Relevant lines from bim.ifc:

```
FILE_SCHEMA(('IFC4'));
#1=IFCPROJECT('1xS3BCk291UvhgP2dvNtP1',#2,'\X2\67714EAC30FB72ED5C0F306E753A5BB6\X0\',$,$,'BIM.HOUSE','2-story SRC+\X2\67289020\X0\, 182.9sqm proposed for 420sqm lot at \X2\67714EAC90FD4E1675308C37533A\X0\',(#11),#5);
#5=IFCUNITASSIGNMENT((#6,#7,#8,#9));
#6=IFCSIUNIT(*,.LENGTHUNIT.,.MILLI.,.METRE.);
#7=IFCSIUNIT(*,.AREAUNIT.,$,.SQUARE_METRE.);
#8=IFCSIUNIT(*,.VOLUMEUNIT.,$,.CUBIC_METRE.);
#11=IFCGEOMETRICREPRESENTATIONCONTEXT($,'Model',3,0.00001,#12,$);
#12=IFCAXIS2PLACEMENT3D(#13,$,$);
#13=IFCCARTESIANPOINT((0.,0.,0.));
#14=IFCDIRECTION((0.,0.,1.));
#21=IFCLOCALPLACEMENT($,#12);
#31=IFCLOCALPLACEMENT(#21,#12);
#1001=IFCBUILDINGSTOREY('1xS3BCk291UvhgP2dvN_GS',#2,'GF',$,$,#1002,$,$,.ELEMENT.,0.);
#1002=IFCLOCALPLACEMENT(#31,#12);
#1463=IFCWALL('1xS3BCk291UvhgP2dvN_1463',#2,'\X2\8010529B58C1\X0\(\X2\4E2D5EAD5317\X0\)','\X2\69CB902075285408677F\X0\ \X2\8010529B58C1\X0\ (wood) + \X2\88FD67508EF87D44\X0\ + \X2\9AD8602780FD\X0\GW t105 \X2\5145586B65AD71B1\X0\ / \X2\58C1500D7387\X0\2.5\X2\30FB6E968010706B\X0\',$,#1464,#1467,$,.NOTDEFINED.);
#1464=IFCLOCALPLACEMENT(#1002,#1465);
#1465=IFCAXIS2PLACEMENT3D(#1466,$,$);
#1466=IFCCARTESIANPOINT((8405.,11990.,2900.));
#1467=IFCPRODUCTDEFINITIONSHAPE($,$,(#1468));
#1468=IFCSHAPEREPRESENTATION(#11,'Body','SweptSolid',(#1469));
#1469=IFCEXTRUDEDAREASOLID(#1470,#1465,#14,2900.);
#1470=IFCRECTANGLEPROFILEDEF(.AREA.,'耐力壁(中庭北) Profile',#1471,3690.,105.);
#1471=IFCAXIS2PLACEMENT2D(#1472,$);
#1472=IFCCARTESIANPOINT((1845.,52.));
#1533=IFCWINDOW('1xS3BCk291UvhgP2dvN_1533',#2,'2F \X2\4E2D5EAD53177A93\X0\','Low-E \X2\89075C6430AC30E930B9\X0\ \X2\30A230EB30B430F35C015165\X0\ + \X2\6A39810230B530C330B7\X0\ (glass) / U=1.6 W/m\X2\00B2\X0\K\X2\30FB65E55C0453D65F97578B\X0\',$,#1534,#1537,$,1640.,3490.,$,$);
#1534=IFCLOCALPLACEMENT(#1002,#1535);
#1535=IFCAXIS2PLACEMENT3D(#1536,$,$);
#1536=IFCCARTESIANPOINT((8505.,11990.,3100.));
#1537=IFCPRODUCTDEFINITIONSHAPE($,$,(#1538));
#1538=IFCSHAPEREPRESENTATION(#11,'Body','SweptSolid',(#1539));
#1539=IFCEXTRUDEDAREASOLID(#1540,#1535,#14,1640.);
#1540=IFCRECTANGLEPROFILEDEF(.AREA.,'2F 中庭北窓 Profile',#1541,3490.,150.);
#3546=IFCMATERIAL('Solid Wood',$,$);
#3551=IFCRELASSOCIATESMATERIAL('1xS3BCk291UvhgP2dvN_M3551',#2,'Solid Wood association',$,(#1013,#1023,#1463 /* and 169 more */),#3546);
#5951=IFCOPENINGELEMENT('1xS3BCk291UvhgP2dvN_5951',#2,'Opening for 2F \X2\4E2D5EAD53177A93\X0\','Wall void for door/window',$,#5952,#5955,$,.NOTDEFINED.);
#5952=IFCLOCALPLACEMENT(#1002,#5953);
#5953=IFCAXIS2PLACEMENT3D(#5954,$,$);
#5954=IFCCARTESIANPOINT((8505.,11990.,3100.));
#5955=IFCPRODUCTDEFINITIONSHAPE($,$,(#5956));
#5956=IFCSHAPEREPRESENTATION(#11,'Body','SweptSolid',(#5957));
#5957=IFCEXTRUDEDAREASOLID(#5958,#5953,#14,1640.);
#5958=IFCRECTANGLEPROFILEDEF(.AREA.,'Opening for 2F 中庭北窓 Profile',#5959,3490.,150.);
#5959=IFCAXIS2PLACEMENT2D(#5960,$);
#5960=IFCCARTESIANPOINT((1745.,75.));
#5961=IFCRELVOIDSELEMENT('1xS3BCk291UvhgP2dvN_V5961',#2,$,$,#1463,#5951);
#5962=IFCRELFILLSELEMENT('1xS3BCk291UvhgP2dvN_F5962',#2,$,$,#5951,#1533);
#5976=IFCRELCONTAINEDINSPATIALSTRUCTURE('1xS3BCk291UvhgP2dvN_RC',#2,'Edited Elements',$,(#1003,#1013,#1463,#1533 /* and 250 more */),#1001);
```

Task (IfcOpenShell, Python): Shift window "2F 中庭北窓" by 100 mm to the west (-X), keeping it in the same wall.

```python
import ifcopenshell
import ifcopenshell.api.geometry
import ifcopenshell.util.placement

model = ifcopenshell.open("bim.ifc")

window = model.by_id(1533)
opening = window.FillsVoids[0].RelatingOpeningElement
wall = opening.VoidsElements[0].RelatingBuildingElement

wall_matrix = ifcopenshell.util.placement.get_local_placement(wall.ObjectPlacement)
shift = wall_matrix[:3, 0] * -100.0
before = ifcopenshell.util.placement.get_local_placement(window.ObjectPlacement)[:3, 3].copy()

# The window is not placed relative to its opening, so move both.
for product in (opening, window):
    matrix = ifcopenshell.util.placement.get_local_placement(product.ObjectPlacement)
    matrix[:3, 3] += shift
    ifcopenshell.api.geometry.edit_object_placement(model, product=product, matrix=matrix, is_si=False)

after = ifcopenshell.util.placement.get_local_placement(window.ObjectPlacement)[:3, 3]
print("window moved by", (after - before).round(3) + 0.0)

model.write("bim-out.ifc")
```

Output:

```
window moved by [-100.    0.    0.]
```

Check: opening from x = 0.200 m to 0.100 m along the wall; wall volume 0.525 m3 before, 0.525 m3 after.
